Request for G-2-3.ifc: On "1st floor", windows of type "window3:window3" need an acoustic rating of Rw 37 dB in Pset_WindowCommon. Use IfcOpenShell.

First a look at what the model holds.

```python
import ifcopenshell
import ifcopenshell.util.element

model = ifcopenshell.open("G-2-3.ifc")
print(model.schema)
storey = next(s for s in model.by_type("IfcBuildingStorey") if s.Name == "1st floor")
windows = [e for e in ifcopenshell.util.element.get_decomposition(storey) if e.is_a("IfcWindow")]
seen = {}
for e in windows:
    element_type = ifcopenshell.util.element.get_type(e)
    key = (element_type.Name if element_type != e and element_type else None, ifcopenshell.util.element.get_pset(e, "Pset_WindowCommon", "AcousticRating"))
    seen[key] = seen.get(key, 0) + 1
for (name, value), count in sorted(seen.items(), key=str):
    print(count, "x", name, "|", value)
```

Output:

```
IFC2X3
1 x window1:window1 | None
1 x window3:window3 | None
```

```python
import ifcopenshell
import ifcopenshell.api.pset
import ifcopenshell.util.element

model = ifcopenshell.open("G-2-3.ifc")

storey = next(s for s in model.by_type("IfcBuildingStorey") if s.Name == "1st floor")
windows = [e for e in ifcopenshell.util.element.get_decomposition(storey) if e.is_a("IfcWindow")]

count = 0
for e in windows:
    element_type = ifcopenshell.util.element.get_type(e)
    if element_type in (None, e) or element_type.Name != "window3:window3":
        continue
    # add_pset returns the element's existing set when there is one.
    pset = ifcopenshell.api.pset.add_pset(model, product=e, name="Pset_WindowCommon")
    ifcopenshell.api.pset.edit_pset(model, pset=pset, properties={"AcousticRating": "Rw 37 dB"})
    count += 1

print(count, "windows updated")

model.write("G-2-3_updated.ifc")
```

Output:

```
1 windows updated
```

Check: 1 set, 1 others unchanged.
